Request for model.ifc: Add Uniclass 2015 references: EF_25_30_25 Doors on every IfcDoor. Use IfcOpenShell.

First a look at what the model holds.

```python
import ifcopenshell

model = ifcopenshell.open("model.ifc")
print(model.schema)
print("classifications:", [c.Name for c in model.by_type("IfcClassification")])
for ifc_class in ("IfcDoor", "IfcRoof", "IfcStair", "IfcWall", "IfcWindow"):
    print(ifc_class, len(model.by_type(ifc_class)))
```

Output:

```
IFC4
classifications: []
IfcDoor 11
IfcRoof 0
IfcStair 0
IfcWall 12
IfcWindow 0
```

```python
import ifcopenshell
import ifcopenshell.api.classification

model = ifcopenshell.open("model.ifc")

system = ifcopenshell.api.classification.add_classification(model, classification="Uniclass 2015")

codes = {
    "IfcDoor": ("EF_25_30_25", "Doors"),
}
for ifc_class, (code, name) in codes.items():
    products = model.by_type(ifc_class)
    ifcopenshell.api.classification.add_reference(
        model, products=products, classification=system, identification=code, name=name
    )
    print(code, len(products))

model.write("model_edited.ifc")
```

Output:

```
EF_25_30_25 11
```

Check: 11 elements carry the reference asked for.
